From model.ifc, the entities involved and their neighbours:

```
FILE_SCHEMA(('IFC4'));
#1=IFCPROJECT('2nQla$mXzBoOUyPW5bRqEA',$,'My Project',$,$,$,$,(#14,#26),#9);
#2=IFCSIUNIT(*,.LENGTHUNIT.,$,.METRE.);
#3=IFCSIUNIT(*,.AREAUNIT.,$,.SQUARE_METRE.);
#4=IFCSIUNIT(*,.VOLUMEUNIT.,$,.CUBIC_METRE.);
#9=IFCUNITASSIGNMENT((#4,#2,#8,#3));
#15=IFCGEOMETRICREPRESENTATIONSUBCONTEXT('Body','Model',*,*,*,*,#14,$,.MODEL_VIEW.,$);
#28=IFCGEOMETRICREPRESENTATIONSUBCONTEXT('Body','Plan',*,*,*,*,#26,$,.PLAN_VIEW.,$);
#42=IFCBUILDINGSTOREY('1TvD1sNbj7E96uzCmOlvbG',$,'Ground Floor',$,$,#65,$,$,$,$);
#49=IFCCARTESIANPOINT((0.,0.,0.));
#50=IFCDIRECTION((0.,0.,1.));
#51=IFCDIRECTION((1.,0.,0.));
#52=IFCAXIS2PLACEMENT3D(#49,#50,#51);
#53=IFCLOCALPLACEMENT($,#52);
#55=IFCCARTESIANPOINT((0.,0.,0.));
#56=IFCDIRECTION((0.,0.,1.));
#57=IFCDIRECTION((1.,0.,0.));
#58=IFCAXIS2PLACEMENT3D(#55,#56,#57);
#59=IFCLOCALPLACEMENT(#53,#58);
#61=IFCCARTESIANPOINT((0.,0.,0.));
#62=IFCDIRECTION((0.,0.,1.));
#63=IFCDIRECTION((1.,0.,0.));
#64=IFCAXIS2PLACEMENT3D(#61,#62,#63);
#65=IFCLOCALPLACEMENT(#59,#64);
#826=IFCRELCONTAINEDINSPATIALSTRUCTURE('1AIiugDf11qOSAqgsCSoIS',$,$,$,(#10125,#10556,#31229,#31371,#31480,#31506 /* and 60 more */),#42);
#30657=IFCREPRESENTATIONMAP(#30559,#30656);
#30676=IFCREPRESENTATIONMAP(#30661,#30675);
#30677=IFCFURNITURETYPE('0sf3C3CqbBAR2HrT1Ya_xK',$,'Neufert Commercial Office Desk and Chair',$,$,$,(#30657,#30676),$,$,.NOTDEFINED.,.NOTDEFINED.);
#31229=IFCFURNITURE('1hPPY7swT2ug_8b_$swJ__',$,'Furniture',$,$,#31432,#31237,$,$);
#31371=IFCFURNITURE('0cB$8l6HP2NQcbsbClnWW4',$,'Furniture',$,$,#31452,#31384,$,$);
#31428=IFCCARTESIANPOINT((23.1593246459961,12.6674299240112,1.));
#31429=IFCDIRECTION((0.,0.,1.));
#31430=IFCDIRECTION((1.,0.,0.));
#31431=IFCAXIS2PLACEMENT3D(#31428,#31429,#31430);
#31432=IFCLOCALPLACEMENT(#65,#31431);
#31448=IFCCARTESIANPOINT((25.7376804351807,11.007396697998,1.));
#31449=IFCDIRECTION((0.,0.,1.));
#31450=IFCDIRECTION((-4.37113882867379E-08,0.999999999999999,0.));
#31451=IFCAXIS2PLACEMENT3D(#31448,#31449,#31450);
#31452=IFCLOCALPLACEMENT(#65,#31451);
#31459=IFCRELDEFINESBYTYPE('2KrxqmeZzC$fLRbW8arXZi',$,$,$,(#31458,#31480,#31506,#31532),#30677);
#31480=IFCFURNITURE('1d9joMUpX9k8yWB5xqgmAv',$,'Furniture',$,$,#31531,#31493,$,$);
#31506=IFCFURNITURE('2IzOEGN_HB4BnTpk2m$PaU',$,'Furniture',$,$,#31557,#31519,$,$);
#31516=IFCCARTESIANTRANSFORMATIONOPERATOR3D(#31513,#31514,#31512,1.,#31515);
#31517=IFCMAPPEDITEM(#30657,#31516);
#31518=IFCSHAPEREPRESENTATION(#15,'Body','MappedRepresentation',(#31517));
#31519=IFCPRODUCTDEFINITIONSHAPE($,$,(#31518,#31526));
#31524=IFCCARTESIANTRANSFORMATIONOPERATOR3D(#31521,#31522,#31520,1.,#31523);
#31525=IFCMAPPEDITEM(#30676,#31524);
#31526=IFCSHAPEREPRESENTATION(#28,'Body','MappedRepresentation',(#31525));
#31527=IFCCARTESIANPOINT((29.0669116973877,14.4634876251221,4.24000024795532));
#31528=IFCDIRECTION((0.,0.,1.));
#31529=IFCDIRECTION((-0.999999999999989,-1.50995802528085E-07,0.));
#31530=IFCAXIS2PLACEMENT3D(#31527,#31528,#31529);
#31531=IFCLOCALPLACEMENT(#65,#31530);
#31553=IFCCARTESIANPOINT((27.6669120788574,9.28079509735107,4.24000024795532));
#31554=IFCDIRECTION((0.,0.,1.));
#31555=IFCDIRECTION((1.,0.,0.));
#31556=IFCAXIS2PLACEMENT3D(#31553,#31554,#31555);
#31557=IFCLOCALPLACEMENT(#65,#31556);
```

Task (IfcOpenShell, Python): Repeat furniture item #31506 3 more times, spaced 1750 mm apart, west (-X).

```python
import numpy as np
import ifcopenshell
import ifcopenshell.api.geometry
import ifcopenshell.api.root
import ifcopenshell.util.element
import ifcopenshell.util.placement

model = ifcopenshell.open("model.ifc")

source = model.by_guid("2IzOEGN_HB4BnTpk2m$PaU")
base = ifcopenshell.util.placement.get_local_placement(source.ObjectPlacement)
step = np.array([-1.0, 0.0, 0.0]) * 1.75

for i in range(1, 4):
    copy = ifcopenshell.api.root.copy_class(model, product=source)
    copy.Representation = ifcopenshell.util.element.copy_deep(
        model, source.Representation, exclude=["IfcGeometricRepresentationContext", "IfcRepresentationMap"]
    )
    matrix = base.copy()
    matrix[:3, 3] += i * step
    print("added at", matrix[:3, 3].round(3) + 0.0)
    ifcopenshell.api.geometry.edit_object_placement(model, product=copy, matrix=matrix, is_si=False)

model.write("model_updated.ifc")
```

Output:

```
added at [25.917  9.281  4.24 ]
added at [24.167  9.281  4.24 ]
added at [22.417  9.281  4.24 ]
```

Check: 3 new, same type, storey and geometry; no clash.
